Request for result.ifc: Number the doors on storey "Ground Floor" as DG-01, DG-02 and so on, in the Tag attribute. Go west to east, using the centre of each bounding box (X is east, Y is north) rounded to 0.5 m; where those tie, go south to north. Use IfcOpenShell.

First a look at what the model holds.

```python
import ifcopenshell
import ifcopenshell.util.element
import ifcopenshell.util.placement

model = ifcopenshell.open("result.ifc")
print(model.schema)
storey = next(s for s in model.by_type("IfcBuildingStorey") if s.Name == "Ground Floor")
doors = [e for e in ifcopenshell.util.element.get_decomposition(storey) if e.is_a("IfcDoor")]
for e in sorted(doors, key=lambda e: e.id()):
    origin = ifcopenshell.util.placement.get_local_placement(e.ObjectPlacement)[:3, 3]
    print(e.id(), e.Tag, e.Name, origin.round(2) + 0.0, sep=" | ")
```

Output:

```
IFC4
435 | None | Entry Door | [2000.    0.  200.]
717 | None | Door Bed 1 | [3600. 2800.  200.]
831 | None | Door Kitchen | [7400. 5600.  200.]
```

```python
import ifcopenshell
import ifcopenshell.geom
import ifcopenshell.util.element
import ifcopenshell.util.shape

model = ifcopenshell.open("result.ifc")
settings = ifcopenshell.geom.settings()
settings.set("use-world-coords", True)


def centre(element):
    shape = ifcopenshell.geom.create_shape(settings, element)
    return ifcopenshell.util.shape.get_bbox_centroid(shape.geometry)


storey = next(s for s in model.by_type("IfcBuildingStorey") if s.Name == "Ground Floor")
doors = [e for e in ifcopenshell.util.element.get_decomposition(storey) if e.is_a("IfcDoor")]

# Insertion points can sit at a corner or the storey origin, so sort by the geometry (in metres).
centres = {e: centre(e) for e in doors}
doors.sort(key=lambda e: (round(centres[e][0] / 0.5), centres[e][1]))

for i, e in enumerate(doors, start=1):
    number = f"DG-{i:02d}"
    e.Tag = number
    print(e.id(), number)

model.write("result_edited.ifc")
```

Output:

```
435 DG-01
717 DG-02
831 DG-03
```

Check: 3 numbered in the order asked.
